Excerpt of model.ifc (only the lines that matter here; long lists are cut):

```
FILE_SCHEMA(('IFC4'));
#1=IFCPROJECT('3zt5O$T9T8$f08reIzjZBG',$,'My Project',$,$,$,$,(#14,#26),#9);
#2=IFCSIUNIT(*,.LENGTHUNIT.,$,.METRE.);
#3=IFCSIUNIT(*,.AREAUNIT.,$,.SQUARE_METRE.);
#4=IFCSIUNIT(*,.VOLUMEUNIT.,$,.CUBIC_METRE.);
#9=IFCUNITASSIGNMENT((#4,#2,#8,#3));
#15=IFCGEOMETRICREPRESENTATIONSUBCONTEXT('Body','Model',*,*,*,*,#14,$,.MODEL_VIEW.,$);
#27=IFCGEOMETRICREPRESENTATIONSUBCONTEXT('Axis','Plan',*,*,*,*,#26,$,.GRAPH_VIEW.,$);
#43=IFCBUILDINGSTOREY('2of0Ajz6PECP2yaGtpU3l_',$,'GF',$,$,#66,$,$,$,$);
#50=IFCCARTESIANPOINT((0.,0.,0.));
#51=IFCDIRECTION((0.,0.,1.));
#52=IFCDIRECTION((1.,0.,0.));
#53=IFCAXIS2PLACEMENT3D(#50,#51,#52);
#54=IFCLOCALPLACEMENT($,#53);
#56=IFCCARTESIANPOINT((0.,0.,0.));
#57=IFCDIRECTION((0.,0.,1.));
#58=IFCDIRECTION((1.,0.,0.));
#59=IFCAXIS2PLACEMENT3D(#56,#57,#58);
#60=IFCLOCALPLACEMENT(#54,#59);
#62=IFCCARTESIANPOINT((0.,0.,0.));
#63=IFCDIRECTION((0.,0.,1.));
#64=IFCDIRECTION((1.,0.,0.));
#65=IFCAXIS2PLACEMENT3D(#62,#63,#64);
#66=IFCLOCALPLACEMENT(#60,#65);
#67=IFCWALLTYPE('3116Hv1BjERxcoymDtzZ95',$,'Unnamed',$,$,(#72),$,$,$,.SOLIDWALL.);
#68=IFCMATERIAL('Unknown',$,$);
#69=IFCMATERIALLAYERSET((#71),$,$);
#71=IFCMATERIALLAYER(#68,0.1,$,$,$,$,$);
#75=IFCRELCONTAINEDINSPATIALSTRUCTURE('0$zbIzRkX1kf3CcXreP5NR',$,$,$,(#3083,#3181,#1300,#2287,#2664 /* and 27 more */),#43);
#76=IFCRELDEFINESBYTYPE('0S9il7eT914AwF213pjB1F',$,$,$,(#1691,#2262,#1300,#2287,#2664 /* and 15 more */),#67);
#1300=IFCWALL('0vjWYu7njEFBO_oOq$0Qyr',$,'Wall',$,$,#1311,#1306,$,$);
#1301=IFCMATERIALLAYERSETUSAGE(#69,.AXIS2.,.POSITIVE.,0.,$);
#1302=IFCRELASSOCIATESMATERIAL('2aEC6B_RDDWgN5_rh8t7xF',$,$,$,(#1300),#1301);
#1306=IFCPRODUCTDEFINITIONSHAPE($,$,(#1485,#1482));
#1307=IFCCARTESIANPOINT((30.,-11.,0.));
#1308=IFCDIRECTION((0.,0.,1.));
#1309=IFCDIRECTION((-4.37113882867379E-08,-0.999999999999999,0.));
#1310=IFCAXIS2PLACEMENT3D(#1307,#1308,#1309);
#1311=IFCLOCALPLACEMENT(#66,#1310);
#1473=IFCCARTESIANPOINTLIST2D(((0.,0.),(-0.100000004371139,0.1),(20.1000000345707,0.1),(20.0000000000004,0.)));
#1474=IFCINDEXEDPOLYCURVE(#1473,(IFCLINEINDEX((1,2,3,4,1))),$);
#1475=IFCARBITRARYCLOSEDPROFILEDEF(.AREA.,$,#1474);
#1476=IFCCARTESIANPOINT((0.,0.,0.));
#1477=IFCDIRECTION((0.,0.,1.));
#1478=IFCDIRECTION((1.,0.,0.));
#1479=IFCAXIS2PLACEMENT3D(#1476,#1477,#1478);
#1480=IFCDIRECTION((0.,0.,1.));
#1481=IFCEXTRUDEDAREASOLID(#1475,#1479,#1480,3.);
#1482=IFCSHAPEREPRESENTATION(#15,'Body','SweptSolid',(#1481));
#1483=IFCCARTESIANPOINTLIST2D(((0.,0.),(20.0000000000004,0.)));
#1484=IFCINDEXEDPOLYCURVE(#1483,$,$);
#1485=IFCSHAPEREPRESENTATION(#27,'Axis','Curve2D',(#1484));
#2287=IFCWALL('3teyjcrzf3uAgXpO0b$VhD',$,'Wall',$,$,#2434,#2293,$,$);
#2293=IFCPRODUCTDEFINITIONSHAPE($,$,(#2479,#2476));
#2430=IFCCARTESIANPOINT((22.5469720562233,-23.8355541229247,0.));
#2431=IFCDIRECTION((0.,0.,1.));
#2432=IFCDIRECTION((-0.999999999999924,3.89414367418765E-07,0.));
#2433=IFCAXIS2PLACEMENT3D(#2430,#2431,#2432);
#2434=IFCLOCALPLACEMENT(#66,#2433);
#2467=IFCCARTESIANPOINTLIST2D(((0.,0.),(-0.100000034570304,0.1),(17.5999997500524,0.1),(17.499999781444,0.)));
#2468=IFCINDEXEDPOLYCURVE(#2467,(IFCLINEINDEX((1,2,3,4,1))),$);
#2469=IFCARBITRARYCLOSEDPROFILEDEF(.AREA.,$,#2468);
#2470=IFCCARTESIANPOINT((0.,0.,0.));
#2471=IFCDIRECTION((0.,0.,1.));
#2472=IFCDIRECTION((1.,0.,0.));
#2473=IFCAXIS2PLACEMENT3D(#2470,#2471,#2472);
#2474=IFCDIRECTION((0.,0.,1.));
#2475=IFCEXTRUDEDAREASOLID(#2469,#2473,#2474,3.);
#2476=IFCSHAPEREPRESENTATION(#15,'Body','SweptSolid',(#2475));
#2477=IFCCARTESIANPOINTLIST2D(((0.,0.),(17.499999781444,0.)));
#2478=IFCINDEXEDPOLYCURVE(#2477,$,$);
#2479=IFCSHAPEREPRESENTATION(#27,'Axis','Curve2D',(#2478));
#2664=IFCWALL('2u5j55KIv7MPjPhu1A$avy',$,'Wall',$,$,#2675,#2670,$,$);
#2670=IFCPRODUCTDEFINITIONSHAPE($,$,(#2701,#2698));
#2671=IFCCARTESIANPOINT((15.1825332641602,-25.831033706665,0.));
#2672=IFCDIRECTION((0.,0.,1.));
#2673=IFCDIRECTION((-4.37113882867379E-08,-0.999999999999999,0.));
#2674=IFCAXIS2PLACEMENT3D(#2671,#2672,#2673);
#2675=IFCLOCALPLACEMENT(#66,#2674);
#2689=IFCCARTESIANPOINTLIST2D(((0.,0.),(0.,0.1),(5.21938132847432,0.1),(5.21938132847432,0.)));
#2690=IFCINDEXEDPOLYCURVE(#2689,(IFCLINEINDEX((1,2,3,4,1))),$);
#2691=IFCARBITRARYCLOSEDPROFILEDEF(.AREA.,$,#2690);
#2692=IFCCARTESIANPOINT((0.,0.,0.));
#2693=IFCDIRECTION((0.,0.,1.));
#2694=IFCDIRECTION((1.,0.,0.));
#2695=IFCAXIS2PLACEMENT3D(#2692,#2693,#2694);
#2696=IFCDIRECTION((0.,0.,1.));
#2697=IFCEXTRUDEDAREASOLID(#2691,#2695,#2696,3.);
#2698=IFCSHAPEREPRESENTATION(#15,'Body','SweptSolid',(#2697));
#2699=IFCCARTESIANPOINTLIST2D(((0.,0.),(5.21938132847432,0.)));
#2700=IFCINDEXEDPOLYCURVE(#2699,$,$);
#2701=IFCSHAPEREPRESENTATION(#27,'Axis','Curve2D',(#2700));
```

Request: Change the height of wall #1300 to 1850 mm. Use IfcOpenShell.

```python
import ifcopenshell
import ifcopenshell.geom
import ifcopenshell.util.representation
import ifcopenshell.util.shape

model = ifcopenshell.open("model.ifc")
settings = ifcopenshell.geom.settings()


def volume(element):
    """Net volume in cubic metres, openings subtracted."""
    shape = ifcopenshell.geom.create_shape(settings, element)
    return ifcopenshell.util.shape.get_volume(shape.geometry)


wall = model.by_guid("0vjWYu7njEFBO_oOq$0Qyr")
before = volume(wall)

body = ifcopenshell.util.representation.get_representation(wall, "Model", "Body")
solid = body.Items[0]
old_height = solid.Depth
solid.Depth = 1.85
after = volume(wall)

print(f"height {old_height:g} -> {solid.Depth:g}, volume {before:.3f} -> {after:.3f} m3")

model.write("model_rev.ifc")
```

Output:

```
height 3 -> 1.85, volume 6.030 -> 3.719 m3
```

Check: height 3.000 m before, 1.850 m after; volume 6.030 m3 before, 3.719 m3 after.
